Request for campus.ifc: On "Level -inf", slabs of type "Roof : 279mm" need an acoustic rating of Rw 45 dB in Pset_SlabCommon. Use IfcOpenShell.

First a look at what the model holds.

```python
import ifcopenshell
import ifcopenshell.util.element

model = ifcopenshell.open("campus.ifc")
print(model.schema)
storey = next(s for s in model.by_type("IfcBuildingStorey") if s.Name == "Level -inf")
slabs = [e for e in ifcopenshell.util.element.get_decomposition(storey) if e.is_a("IfcSlab")]
seen = {}
for e in slabs:
    element_type = ifcopenshell.util.element.get_type(e)
    key = (element_type.Name if element_type != e and element_type else None, ifcopenshell.util.element.get_pset(e, "Pset_SlabCommon", "AcousticRating"))
    seen[key] = seen.get(key, 0) + 1
for (name, value), count in sorted(seen.items(), key=str):
    print(count, "x", name, "|", value)
```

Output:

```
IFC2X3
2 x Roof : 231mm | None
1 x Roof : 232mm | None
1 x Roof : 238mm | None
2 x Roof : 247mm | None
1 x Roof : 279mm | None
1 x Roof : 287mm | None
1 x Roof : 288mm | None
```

```python
import ifcopenshell
import ifcopenshell.api.pset
import ifcopenshell.util.element

model = ifcopenshell.open("campus.ifc")

storey = next(s for s in model.by_type("IfcBuildingStorey") if s.Name == "Level -inf")
slabs = [e for e in ifcopenshell.util.element.get_decomposition(storey) if e.is_a("IfcSlab")]

count = 0
for e in slabs:
    element_type = ifcopenshell.util.element.get_type(e)
    if element_type in (None, e) or element_type.Name != "Roof : 279mm":
        continue
    # add_pset returns the element's existing set when there is one.
    pset = ifcopenshell.api.pset.add_pset(model, product=e, name="Pset_SlabCommon")
    ifcopenshell.api.pset.edit_pset(model, pset=pset, properties={"AcousticRating": "Rw 45 dB"})
    count += 1

print(count, "slabs updated")

model.write("campus_updated.ifc")
```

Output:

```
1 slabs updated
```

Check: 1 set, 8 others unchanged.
